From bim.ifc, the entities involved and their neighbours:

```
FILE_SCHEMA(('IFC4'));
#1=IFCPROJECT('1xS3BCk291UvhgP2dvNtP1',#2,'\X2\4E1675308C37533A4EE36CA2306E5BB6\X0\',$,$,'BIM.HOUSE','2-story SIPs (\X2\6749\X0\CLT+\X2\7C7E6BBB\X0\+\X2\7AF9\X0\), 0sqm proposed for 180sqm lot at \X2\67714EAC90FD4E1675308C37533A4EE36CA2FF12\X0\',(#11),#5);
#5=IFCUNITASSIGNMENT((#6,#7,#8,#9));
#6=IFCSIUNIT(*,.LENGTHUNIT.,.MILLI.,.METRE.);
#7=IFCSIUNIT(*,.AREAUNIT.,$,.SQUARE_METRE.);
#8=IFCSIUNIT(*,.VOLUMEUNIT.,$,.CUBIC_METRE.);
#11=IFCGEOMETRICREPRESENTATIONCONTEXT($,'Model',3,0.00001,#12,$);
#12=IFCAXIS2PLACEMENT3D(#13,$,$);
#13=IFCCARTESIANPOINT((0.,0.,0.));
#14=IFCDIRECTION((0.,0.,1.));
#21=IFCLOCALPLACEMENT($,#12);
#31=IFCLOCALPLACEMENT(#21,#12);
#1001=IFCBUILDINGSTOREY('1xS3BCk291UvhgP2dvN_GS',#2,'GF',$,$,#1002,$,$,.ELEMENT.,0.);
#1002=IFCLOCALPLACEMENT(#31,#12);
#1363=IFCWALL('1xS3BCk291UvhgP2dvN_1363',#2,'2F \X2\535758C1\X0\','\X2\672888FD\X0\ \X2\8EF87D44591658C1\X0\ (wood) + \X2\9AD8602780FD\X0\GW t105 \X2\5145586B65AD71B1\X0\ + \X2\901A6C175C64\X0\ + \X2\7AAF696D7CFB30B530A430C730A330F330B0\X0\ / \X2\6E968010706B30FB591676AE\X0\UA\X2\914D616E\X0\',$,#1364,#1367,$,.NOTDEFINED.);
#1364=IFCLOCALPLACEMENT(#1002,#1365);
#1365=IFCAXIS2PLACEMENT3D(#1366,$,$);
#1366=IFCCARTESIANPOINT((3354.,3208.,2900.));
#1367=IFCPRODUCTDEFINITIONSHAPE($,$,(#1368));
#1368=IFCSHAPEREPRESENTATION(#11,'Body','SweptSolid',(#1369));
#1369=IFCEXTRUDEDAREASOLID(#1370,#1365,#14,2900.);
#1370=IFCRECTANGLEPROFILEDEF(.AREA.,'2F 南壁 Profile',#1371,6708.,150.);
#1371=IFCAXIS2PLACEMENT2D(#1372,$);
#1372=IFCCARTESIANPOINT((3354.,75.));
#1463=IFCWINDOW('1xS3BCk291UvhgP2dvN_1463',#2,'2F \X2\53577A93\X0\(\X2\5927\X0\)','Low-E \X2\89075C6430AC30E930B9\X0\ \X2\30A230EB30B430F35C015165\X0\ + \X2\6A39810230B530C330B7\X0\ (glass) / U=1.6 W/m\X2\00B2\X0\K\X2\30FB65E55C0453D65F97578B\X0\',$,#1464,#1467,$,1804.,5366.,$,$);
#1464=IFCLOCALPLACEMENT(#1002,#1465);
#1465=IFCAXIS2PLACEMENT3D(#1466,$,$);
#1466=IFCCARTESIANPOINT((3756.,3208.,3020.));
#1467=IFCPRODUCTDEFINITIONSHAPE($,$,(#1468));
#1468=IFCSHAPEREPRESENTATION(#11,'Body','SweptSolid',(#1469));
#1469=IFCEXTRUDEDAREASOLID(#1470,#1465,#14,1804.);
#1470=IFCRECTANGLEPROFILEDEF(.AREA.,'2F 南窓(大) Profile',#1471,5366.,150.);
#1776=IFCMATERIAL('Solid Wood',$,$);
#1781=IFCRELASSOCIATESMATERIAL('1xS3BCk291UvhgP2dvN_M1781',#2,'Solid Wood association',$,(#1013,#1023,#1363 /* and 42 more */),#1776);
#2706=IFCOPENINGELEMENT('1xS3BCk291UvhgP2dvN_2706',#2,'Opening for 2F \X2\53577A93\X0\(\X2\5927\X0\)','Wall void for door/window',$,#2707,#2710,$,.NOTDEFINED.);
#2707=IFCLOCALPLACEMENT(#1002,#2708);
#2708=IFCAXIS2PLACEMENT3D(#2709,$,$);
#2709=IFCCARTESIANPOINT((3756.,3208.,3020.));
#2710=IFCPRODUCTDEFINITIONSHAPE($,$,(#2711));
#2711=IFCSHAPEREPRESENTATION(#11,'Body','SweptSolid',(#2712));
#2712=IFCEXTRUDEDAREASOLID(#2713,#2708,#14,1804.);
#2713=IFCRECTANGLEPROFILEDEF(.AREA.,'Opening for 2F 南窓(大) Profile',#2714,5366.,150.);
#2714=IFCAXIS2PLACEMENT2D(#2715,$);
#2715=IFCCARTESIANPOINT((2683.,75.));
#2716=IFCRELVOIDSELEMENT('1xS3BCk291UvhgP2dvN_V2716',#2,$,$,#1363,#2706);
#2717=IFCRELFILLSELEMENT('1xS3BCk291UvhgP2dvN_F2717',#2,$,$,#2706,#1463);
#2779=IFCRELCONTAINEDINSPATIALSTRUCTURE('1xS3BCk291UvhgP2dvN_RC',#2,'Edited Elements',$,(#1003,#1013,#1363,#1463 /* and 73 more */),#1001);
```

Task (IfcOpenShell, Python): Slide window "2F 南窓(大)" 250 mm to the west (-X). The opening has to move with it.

```python
import ifcopenshell
import ifcopenshell.api.geometry
import ifcopenshell.util.placement
import ifcopenshell.util.unit

model = ifcopenshell.open("bim.ifc")
unit_scale = ifcopenshell.util.unit.calculate_unit_scale(model)

window = model.by_guid("1xS3BCk291UvhgP2dvN_1463")
opening = window.FillsVoids[0].RelatingOpeningElement
wall = opening.VoidsElements[0].RelatingBuildingElement

wall_matrix = ifcopenshell.util.placement.get_local_placement(wall.ObjectPlacement)
shift = wall_matrix[:3, 0] * -0.25 / unit_scale
before = ifcopenshell.util.placement.get_local_placement(window.ObjectPlacement)[:3, 3].copy()

# The window is not placed relative to its opening, so move both.
for product in (opening, window):
    matrix = ifcopenshell.util.placement.get_local_placement(product.ObjectPlacement)
    matrix[:3, 3] += shift
    ifcopenshell.api.geometry.edit_object_placement(model, product=product, matrix=matrix, is_si=False)

after = ifcopenshell.util.placement.get_local_placement(window.ObjectPlacement)[:3, 3]
print("window moved by", (after - before).round(3) + 0.0)

model.write("bim_updated.ifc")
```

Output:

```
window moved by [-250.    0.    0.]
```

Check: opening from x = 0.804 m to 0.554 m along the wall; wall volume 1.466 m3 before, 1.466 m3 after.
